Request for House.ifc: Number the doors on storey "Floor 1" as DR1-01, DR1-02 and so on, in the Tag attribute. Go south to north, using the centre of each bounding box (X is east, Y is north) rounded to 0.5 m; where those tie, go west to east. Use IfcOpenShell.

First a look at what the model holds.

```python
import ifcopenshell
import ifcopenshell.util.element
import ifcopenshell.util.placement

model = ifcopenshell.open("House.ifc")
print(model.schema)
storey = next(s for s in model.by_type("IfcBuildingStorey") if s.Name == "Floor 1")
doors = [e for e in ifcopenshell.util.element.get_decomposition(storey) if e.is_a("IfcDoor")]
for e in sorted(doors, key=lambda e: e.id()):
    origin = ifcopenshell.util.placement.get_local_placement(e.ObjectPlacement)[:3, 3]
    print(e.id(), e.Tag, e.Name, origin.round(2) + 0.0, sep=" | ")
```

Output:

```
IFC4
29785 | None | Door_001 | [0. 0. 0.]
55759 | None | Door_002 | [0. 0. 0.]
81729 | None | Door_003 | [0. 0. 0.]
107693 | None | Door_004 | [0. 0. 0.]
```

```python
import ifcopenshell
import ifcopenshell.geom
import ifcopenshell.util.element
import ifcopenshell.util.shape

model = ifcopenshell.open("House.ifc")
settings = ifcopenshell.geom.settings()
settings.set("use-world-coords", True)


def centre(element):
    shape = ifcopenshell.geom.create_shape(settings, element)
    return ifcopenshell.util.shape.get_bbox_centroid(shape.geometry)


storey = next(s for s in model.by_type("IfcBuildingStorey") if s.Name == "Floor 1")
doors = [e for e in ifcopenshell.util.element.get_decomposition(storey) if e.is_a("IfcDoor")]

# Insertion points can sit at a corner or the storey origin, so sort by the geometry (in metres).
centres = {e: centre(e) for e in doors}
doors.sort(key=lambda e: (round(centres[e][1] / 0.5), centres[e][0]))

for i, e in enumerate(doors, start=1):
    number = f"DR1-{i:02d}"
    e.Tag = number
    print(e.id(), number)

model.write("House-out.ifc")
```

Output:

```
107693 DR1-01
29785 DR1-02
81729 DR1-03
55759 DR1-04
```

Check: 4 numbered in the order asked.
